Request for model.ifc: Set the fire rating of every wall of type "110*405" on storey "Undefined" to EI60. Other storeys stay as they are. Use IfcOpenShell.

First a look at what the model holds.

```python
import ifcopenshell
import ifcopenshell.util.element

model = ifcopenshell.open("model.ifc")
print(model.schema)
storey = next(s for s in model.by_type("IfcBuildingStorey") if s.Name == "Undefined")
walls = [e for e in ifcopenshell.util.element.get_decomposition(storey) if e.is_a("IfcWall")]
seen = {}
for e in walls:
    element_type = ifcopenshell.util.element.get_type(e)
    key = (element_type.Name if element_type != e and element_type else None, ifcopenshell.util.element.get_pset(e, "Pset_WallCommon", "FireRating"))
    seen[key] = seen.get(key, 0) + 1
for (name, value), count in sorted(seen.items(), key=str):
    print(count, "x", name, "|", value)
```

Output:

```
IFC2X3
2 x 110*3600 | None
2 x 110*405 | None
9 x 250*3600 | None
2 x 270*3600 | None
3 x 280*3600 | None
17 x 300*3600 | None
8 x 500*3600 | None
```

```python
import ifcopenshell
import ifcopenshell.api.pset
import ifcopenshell.util.element

model = ifcopenshell.open("model.ifc")

storey = next(s for s in model.by_type("IfcBuildingStorey") if s.Name == "Undefined")
walls = [e for e in ifcopenshell.util.element.get_decomposition(storey) if e.is_a("IfcWall")]

count = 0
for e in walls:
    element_type = ifcopenshell.util.element.get_type(e)
    if element_type in (None, e) or element_type.Name != "110*405":
        continue
    found = ifcopenshell.util.element.get_pset(e, "Pset_WallCommon", should_inherit=False)
    if found:
        pset = model.by_id(found["id"])
        if len(ifcopenshell.util.element.get_elements_by_pset(pset)) > 1:
            pset = ifcopenshell.api.pset.unshare_pset(model, products=[e], pset=pset)[0]
    else:
        pset = ifcopenshell.api.pset.add_pset(model, product=e, name="Pset_WallCommon")
    ifcopenshell.api.pset.edit_pset(model, pset=pset, properties={"FireRating": "EI60"})
    count += 1

print(count, "walls updated")

model.write("model_rev.ifc")
```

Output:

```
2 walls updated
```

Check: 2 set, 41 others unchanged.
